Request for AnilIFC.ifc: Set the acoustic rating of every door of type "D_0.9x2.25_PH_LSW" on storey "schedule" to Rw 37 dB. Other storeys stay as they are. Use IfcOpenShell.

First a look at what the model holds.

```python
import ifcopenshell
import ifcopenshell.util.element

model = ifcopenshell.open("AnilIFC.ifc")
print(model.schema)
storey = next(s for s in model.by_type("IfcBuildingStorey") if s.Name == "schedule")
doors = [e for e in ifcopenshell.util.element.get_decomposition(storey) if e.is_a("IfcDoor")]
seen = {}
for e in doors:
    element_type = ifcopenshell.util.element.get_type(e)
    key = (element_type.Name if element_type != e and element_type else None, ifcopenshell.util.element.get_pset(e, "Pset_DoorCommon", "AcousticRating"))
    seen[key] = seen.get(key, 0) + 1
for (name, value), count in sorted(seen.items(), key=str):
    print(count, "x", name, "|", value)
```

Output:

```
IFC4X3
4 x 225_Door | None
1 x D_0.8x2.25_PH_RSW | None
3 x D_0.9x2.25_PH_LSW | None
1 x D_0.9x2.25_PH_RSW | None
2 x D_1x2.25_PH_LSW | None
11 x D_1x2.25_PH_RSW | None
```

```python
import ifcopenshell
import ifcopenshell.api.pset
import ifcopenshell.util.element

model = ifcopenshell.open("AnilIFC.ifc")

storey = next(s for s in model.by_type("IfcBuildingStorey") if s.Name == "schedule")
doors = [e for e in ifcopenshell.util.element.get_decomposition(storey) if e.is_a("IfcDoor")]

count = 0
for e in doors:
    element_type = ifcopenshell.util.element.get_type(e)
    if element_type in (None, e) or element_type.Name != "D_0.9x2.25_PH_LSW":
        continue
    # add_pset returns the element's existing set when there is one.
    pset = ifcopenshell.api.pset.add_pset(model, product=e, name="Pset_DoorCommon")
    ifcopenshell.api.pset.edit_pset(model, pset=pset, properties={"AcousticRating": "Rw 37 dB"})
    count += 1

print(count, "doors updated")

model.write("AnilIFC-out.ifc")
```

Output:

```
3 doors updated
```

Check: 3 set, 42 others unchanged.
